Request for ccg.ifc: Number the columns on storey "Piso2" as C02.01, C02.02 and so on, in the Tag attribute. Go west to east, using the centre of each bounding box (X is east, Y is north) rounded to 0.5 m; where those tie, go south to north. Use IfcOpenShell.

First a look at what the model holds.

```python
import ifcopenshell
import ifcopenshell.util.element
import ifcopenshell.util.placement

model = ifcopenshell.open("ccg.ifc")
print(model.schema)
storey = next(s for s in model.by_type("IfcBuildingStorey") if s.Name == "Piso2")
columns = [e for e in ifcopenshell.util.element.get_decomposition(storey) if e.is_a("IfcColumn")]
for e in sorted(columns, key=lambda e: e.id()):
    origin = ifcopenshell.util.placement.get_local_placement(e.ObjectPlacement)[:3, 3]
    print(e.id(), e.Tag, e.Name, origin.round(2) + 0.0, sep=" | ")
```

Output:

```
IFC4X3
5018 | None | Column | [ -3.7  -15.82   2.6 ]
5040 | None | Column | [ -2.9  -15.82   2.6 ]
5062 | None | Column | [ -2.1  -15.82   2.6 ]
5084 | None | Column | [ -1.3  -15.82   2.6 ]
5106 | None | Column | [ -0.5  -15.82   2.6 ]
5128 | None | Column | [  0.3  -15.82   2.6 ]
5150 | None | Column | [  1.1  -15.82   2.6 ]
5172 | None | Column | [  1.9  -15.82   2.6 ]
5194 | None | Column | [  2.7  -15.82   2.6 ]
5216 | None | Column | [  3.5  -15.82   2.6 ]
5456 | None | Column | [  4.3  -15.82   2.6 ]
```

```python
import ifcopenshell
import ifcopenshell.geom
import ifcopenshell.util.element
import ifcopenshell.util.shape

model = ifcopenshell.open("ccg.ifc")
settings = ifcopenshell.geom.settings()
settings.set("use-world-coords", True)


def centre(element):
    shape = ifcopenshell.geom.create_shape(settings, element)
    return ifcopenshell.util.shape.get_bbox_centroid(shape.geometry)


storey = next(s for s in model.by_type("IfcBuildingStorey") if s.Name == "Piso2")
columns = [e for e in ifcopenshell.util.element.get_decomposition(storey) if e.is_a("IfcColumn")]

# Insertion points can sit at a corner or the storey origin, so sort by the geometry (in metres).
centres = {e: centre(e) for e in columns}
columns.sort(key=lambda e: (round(centres[e][0] / 0.5), centres[e][1]))

for i, e in enumerate(columns, start=1):
    number = f"C02.{i:02d}"
    e.Tag = number
    print(e.id(), number)

model.write("ccg_updated.ifc")
```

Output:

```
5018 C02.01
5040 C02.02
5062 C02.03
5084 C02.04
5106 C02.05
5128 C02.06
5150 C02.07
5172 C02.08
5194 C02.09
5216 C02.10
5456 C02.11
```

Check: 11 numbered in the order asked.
